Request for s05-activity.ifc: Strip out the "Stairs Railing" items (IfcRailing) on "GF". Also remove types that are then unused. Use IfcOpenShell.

First a look at what the model holds.

```python
import ifcopenshell
import ifcopenshell.util.element

model = ifcopenshell.open("s05-activity.ifc")
print(model.schema)
storey = next(s for s in model.by_type("IfcBuildingStorey") if s.Name == "GF")
railings = [e for e in ifcopenshell.util.element.get_decomposition(storey) if e.is_a("IfcRailing")]
seen = {}
for e in railings:
    element_type = ifcopenshell.util.element.get_type(e)
    name = element_type.Name if element_type not in (None, e) else None
    seen[name] = seen.get(name, 0) + 1
for name, count in sorted(seen.items(), key=str):
    print(count, "x", name)
```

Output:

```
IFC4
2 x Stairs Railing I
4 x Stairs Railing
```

```python
import ifcopenshell
import ifcopenshell.api.root
import ifcopenshell.util.element

model = ifcopenshell.open("s05-activity.ifc")

storey = next(s for s in model.by_type("IfcBuildingStorey") if s.Name == "GF")
railings = [e for e in ifcopenshell.util.element.get_decomposition(storey) if e.is_a("IfcRailing")]
targets = [e for e in railings if (t := ifcopenshell.util.element.get_type(e)) not in (None, e) and t.Name == "Stairs Railing"]
types = {ifcopenshell.util.element.get_type(e) for e in targets} - {None, *targets}

for e in targets:
    ifcopenshell.api.root.remove_product(model, product=e)
print(len(targets), "removed")

unused = [t for t in types if not ifcopenshell.util.element.get_types(t)]
for t in unused:
    ifcopenshell.api.root.remove_product(model, product=t)
print(len(unused), "unused types removed")

model.write("s05-activity_rev.ifc")
```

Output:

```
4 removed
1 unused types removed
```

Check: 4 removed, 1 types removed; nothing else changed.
